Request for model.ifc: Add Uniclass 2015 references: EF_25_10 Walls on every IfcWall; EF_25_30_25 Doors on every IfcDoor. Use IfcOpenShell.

First a look at what the model holds.

```python
import ifcopenshell

model = ifcopenshell.open("model.ifc")
print(model.schema)
print("classifications:", [c.Name for c in model.by_type("IfcClassification")])
for ifc_class in ("IfcDoor", "IfcRoof", "IfcStair", "IfcWall", "IfcWindow"):
    print(ifc_class, len(model.by_type(ifc_class)))
```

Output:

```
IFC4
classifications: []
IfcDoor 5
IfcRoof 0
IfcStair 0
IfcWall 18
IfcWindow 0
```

```python
import ifcopenshell
import ifcopenshell.api.classification

model = ifcopenshell.open("model.ifc")

system = ifcopenshell.api.classification.add_classification(model, classification="Uniclass 2015")

codes = {
    "IfcWall": ("EF_25_10", "Walls"),
    "IfcDoor": ("EF_25_30_25", "Doors"),
}
for ifc_class, (code, name) in codes.items():
    products = model.by_type(ifc_class)
    ifcopenshell.api.classification.add_reference(
        model, products=products, classification=system, identification=code, name=name
    )
    print(code, len(products))

model.write("model_v2.ifc")
```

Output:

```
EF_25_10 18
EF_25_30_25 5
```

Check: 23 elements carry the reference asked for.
